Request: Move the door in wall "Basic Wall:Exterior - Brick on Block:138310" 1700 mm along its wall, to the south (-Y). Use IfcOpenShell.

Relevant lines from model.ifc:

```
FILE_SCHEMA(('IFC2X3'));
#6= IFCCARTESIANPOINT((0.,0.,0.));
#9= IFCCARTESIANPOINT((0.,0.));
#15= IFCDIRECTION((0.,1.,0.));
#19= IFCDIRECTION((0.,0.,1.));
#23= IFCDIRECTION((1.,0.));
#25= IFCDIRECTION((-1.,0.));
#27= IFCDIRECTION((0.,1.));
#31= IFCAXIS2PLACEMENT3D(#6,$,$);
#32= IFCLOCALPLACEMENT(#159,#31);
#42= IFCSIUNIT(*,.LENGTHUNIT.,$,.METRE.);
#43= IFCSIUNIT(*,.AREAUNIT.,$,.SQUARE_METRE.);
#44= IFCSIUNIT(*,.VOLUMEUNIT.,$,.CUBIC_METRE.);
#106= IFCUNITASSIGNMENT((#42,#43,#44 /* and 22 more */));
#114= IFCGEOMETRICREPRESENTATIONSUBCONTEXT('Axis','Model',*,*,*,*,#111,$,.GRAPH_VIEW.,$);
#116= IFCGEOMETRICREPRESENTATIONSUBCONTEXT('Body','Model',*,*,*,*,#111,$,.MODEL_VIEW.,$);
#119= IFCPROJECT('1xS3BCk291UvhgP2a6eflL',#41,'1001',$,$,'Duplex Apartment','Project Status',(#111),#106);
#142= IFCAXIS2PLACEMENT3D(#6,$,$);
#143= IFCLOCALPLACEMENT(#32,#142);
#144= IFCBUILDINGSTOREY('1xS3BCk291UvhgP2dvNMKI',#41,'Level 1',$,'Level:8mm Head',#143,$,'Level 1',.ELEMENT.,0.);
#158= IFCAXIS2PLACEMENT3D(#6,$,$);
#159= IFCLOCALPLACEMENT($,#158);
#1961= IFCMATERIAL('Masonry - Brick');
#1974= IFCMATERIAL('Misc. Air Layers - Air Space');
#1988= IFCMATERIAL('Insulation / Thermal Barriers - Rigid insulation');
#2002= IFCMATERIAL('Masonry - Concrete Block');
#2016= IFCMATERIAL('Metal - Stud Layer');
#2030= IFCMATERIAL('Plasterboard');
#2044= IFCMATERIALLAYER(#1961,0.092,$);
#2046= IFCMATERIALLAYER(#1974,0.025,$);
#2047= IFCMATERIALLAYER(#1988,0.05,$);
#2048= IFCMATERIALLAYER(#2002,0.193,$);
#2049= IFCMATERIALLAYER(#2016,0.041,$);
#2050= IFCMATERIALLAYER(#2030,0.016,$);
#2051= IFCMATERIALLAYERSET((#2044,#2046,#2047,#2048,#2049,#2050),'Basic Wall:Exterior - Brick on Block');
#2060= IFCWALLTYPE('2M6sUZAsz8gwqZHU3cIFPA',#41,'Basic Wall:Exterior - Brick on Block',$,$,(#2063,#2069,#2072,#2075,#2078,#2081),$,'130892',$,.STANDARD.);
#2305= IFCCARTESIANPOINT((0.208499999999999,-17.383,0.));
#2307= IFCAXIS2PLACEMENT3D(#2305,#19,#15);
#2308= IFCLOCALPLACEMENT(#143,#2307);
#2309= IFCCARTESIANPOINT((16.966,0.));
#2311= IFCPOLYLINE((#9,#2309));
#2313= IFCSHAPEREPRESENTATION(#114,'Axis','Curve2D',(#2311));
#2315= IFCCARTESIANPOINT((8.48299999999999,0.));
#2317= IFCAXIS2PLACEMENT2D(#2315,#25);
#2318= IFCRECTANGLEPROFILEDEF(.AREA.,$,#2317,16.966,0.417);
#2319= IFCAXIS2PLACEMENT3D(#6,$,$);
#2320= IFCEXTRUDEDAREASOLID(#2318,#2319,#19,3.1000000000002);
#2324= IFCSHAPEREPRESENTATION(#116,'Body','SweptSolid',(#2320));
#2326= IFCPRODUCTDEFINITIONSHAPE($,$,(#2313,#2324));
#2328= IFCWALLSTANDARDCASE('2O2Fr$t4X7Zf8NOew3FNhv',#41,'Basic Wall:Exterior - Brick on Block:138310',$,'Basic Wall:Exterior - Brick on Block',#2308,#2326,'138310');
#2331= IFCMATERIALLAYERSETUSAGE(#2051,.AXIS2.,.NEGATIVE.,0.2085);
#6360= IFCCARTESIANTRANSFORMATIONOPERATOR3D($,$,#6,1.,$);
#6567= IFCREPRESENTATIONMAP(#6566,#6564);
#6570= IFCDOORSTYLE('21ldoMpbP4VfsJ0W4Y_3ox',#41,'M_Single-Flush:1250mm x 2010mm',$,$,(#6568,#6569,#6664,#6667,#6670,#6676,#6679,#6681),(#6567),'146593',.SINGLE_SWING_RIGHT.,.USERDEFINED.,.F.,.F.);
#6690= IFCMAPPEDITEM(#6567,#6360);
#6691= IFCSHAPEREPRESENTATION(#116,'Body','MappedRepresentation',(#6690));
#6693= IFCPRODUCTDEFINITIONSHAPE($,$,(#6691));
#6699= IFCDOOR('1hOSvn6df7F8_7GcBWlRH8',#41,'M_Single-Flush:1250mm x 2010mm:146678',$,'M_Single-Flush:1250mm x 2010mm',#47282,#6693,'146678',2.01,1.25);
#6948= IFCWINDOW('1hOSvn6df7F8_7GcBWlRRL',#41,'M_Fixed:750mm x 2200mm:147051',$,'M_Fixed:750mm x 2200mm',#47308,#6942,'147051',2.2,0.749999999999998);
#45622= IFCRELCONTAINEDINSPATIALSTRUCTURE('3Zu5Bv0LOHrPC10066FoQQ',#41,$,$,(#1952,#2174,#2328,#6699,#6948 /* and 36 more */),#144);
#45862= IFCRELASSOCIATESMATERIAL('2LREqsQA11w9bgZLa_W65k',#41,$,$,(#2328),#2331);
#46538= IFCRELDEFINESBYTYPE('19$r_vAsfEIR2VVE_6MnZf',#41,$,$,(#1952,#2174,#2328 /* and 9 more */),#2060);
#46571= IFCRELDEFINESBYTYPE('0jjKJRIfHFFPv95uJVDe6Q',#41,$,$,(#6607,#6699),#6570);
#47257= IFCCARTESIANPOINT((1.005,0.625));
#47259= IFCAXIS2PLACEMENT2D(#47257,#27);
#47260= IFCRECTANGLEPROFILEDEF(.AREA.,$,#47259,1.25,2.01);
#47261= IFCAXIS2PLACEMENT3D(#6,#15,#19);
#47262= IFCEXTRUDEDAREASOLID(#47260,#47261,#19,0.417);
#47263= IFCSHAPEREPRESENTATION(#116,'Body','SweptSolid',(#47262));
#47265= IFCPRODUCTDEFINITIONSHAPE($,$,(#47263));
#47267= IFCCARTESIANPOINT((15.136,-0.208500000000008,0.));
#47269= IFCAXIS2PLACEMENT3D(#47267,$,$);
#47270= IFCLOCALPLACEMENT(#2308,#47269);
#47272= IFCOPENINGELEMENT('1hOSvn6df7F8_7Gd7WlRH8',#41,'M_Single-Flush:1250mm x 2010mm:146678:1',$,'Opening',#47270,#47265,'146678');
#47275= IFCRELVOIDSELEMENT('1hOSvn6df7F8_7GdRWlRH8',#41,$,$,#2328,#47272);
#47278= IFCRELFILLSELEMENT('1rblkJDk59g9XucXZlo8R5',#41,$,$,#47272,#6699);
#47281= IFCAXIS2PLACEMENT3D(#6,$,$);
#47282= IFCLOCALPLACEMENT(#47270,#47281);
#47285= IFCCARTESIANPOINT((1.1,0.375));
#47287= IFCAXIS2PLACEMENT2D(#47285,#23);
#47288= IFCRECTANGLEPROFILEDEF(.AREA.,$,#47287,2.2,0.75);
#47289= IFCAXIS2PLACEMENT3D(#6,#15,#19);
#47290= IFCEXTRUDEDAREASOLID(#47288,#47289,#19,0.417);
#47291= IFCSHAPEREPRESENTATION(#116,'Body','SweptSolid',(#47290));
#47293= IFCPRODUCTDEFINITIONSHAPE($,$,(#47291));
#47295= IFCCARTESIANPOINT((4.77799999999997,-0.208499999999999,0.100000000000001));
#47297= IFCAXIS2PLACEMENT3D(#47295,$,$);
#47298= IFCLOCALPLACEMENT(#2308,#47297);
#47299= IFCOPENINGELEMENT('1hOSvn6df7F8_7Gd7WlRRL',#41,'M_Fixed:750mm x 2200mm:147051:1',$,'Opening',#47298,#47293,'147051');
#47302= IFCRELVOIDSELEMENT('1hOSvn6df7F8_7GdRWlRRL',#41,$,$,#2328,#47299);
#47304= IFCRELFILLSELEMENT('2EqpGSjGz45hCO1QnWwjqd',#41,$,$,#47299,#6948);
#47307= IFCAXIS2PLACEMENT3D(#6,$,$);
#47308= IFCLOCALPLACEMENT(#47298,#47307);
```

```python
import ifcopenshell
import ifcopenshell.api.geometry
import ifcopenshell.util.placement

model = ifcopenshell.open("model.ifc")

door = model.by_id(6699)
opening = door.FillsVoids[0].RelatingOpeningElement
wall = opening.VoidsElements[0].RelatingBuildingElement

wall_matrix = ifcopenshell.util.placement.get_local_placement(wall.ObjectPlacement)
shift = wall_matrix[:3, 0] * -1.7
before = ifcopenshell.util.placement.get_local_placement(door.ObjectPlacement)[:3, 3].copy()

# The door is placed relative to its opening, so it follows when the opening moves.
matrix = ifcopenshell.util.placement.get_local_placement(opening.ObjectPlacement)
matrix[:3, 3] += shift
ifcopenshell.api.geometry.edit_object_placement(
    model, product=opening, matrix=matrix, is_si=False, should_transform_children=True
)

after = ifcopenshell.util.placement.get_local_placement(door.ObjectPlacement)[:3, 3]
print("door moved by", (after - before).round(3) + 0.0)

model.write("model_updated.ifc")
```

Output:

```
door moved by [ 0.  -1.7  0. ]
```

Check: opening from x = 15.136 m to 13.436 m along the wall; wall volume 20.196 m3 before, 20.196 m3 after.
